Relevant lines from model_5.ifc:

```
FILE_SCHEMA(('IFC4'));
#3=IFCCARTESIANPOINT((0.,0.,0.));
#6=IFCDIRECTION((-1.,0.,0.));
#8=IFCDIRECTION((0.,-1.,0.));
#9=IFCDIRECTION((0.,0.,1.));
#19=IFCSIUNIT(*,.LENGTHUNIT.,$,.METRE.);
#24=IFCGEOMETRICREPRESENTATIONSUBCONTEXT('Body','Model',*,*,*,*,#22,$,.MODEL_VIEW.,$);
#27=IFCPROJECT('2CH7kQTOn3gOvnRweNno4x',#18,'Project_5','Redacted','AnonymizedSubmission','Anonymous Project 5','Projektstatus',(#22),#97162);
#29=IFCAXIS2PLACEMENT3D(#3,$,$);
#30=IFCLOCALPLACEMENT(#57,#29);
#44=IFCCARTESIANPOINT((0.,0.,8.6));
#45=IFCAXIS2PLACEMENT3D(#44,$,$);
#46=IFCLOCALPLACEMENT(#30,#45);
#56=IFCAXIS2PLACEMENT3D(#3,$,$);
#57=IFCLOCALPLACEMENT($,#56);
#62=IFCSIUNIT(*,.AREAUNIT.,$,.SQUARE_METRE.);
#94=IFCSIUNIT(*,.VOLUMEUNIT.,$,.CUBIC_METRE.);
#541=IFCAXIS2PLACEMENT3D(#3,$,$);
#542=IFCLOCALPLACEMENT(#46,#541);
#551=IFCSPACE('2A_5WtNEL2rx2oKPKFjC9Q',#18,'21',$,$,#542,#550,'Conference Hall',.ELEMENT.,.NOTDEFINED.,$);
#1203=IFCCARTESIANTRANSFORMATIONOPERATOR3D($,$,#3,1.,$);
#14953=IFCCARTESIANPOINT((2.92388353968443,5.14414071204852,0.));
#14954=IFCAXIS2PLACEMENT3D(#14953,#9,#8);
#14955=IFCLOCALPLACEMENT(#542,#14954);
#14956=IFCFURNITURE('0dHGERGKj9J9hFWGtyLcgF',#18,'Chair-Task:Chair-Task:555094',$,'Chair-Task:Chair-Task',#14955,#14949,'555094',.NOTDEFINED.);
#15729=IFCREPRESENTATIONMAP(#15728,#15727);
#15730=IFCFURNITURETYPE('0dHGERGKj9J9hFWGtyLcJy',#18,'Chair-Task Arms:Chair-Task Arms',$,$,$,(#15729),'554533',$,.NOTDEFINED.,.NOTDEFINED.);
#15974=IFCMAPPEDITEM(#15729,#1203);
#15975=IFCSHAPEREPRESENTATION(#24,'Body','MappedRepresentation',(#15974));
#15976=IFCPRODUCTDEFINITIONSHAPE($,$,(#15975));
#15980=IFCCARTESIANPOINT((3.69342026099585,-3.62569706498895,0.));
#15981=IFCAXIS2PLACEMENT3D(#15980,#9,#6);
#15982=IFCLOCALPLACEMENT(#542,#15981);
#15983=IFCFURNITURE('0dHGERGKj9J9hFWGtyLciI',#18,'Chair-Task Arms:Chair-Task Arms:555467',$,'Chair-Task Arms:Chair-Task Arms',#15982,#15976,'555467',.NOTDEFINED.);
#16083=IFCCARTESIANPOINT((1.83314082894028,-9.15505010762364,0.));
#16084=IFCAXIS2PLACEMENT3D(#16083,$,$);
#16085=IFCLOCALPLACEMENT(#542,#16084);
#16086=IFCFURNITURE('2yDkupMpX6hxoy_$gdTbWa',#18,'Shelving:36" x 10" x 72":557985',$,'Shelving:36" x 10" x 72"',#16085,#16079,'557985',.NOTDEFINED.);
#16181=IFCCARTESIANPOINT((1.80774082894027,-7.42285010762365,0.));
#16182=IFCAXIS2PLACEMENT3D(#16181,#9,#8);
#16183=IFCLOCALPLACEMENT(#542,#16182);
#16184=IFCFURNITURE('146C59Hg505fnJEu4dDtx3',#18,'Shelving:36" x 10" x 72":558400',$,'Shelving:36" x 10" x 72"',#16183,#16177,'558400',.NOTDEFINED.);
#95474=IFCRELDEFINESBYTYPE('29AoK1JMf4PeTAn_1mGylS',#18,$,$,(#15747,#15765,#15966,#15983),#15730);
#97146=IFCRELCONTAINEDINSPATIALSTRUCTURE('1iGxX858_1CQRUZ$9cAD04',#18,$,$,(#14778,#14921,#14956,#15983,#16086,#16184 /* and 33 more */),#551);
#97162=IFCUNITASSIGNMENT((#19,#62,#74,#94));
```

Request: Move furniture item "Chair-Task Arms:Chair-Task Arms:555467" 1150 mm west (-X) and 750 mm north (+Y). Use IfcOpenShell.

```python
import ifcopenshell
import ifcopenshell.api.geometry
import ifcopenshell.util.placement

model = ifcopenshell.open("model_5.ifc")

item = model.by_id(15983)
matrix = ifcopenshell.util.placement.get_local_placement(item.ObjectPlacement)
matrix[0, 3] -= 1.15
matrix[1, 3] += 0.75
ifcopenshell.api.geometry.edit_object_placement(model, product=item, matrix=matrix, is_si=False)

print(ifcopenshell.util.placement.get_local_placement(item.ObjectPlacement).round(3) + 0.0)

model.write("model_5-out.ifc")
```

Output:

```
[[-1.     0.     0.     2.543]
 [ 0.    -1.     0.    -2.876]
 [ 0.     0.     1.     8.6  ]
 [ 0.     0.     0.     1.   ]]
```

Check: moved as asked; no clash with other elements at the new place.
